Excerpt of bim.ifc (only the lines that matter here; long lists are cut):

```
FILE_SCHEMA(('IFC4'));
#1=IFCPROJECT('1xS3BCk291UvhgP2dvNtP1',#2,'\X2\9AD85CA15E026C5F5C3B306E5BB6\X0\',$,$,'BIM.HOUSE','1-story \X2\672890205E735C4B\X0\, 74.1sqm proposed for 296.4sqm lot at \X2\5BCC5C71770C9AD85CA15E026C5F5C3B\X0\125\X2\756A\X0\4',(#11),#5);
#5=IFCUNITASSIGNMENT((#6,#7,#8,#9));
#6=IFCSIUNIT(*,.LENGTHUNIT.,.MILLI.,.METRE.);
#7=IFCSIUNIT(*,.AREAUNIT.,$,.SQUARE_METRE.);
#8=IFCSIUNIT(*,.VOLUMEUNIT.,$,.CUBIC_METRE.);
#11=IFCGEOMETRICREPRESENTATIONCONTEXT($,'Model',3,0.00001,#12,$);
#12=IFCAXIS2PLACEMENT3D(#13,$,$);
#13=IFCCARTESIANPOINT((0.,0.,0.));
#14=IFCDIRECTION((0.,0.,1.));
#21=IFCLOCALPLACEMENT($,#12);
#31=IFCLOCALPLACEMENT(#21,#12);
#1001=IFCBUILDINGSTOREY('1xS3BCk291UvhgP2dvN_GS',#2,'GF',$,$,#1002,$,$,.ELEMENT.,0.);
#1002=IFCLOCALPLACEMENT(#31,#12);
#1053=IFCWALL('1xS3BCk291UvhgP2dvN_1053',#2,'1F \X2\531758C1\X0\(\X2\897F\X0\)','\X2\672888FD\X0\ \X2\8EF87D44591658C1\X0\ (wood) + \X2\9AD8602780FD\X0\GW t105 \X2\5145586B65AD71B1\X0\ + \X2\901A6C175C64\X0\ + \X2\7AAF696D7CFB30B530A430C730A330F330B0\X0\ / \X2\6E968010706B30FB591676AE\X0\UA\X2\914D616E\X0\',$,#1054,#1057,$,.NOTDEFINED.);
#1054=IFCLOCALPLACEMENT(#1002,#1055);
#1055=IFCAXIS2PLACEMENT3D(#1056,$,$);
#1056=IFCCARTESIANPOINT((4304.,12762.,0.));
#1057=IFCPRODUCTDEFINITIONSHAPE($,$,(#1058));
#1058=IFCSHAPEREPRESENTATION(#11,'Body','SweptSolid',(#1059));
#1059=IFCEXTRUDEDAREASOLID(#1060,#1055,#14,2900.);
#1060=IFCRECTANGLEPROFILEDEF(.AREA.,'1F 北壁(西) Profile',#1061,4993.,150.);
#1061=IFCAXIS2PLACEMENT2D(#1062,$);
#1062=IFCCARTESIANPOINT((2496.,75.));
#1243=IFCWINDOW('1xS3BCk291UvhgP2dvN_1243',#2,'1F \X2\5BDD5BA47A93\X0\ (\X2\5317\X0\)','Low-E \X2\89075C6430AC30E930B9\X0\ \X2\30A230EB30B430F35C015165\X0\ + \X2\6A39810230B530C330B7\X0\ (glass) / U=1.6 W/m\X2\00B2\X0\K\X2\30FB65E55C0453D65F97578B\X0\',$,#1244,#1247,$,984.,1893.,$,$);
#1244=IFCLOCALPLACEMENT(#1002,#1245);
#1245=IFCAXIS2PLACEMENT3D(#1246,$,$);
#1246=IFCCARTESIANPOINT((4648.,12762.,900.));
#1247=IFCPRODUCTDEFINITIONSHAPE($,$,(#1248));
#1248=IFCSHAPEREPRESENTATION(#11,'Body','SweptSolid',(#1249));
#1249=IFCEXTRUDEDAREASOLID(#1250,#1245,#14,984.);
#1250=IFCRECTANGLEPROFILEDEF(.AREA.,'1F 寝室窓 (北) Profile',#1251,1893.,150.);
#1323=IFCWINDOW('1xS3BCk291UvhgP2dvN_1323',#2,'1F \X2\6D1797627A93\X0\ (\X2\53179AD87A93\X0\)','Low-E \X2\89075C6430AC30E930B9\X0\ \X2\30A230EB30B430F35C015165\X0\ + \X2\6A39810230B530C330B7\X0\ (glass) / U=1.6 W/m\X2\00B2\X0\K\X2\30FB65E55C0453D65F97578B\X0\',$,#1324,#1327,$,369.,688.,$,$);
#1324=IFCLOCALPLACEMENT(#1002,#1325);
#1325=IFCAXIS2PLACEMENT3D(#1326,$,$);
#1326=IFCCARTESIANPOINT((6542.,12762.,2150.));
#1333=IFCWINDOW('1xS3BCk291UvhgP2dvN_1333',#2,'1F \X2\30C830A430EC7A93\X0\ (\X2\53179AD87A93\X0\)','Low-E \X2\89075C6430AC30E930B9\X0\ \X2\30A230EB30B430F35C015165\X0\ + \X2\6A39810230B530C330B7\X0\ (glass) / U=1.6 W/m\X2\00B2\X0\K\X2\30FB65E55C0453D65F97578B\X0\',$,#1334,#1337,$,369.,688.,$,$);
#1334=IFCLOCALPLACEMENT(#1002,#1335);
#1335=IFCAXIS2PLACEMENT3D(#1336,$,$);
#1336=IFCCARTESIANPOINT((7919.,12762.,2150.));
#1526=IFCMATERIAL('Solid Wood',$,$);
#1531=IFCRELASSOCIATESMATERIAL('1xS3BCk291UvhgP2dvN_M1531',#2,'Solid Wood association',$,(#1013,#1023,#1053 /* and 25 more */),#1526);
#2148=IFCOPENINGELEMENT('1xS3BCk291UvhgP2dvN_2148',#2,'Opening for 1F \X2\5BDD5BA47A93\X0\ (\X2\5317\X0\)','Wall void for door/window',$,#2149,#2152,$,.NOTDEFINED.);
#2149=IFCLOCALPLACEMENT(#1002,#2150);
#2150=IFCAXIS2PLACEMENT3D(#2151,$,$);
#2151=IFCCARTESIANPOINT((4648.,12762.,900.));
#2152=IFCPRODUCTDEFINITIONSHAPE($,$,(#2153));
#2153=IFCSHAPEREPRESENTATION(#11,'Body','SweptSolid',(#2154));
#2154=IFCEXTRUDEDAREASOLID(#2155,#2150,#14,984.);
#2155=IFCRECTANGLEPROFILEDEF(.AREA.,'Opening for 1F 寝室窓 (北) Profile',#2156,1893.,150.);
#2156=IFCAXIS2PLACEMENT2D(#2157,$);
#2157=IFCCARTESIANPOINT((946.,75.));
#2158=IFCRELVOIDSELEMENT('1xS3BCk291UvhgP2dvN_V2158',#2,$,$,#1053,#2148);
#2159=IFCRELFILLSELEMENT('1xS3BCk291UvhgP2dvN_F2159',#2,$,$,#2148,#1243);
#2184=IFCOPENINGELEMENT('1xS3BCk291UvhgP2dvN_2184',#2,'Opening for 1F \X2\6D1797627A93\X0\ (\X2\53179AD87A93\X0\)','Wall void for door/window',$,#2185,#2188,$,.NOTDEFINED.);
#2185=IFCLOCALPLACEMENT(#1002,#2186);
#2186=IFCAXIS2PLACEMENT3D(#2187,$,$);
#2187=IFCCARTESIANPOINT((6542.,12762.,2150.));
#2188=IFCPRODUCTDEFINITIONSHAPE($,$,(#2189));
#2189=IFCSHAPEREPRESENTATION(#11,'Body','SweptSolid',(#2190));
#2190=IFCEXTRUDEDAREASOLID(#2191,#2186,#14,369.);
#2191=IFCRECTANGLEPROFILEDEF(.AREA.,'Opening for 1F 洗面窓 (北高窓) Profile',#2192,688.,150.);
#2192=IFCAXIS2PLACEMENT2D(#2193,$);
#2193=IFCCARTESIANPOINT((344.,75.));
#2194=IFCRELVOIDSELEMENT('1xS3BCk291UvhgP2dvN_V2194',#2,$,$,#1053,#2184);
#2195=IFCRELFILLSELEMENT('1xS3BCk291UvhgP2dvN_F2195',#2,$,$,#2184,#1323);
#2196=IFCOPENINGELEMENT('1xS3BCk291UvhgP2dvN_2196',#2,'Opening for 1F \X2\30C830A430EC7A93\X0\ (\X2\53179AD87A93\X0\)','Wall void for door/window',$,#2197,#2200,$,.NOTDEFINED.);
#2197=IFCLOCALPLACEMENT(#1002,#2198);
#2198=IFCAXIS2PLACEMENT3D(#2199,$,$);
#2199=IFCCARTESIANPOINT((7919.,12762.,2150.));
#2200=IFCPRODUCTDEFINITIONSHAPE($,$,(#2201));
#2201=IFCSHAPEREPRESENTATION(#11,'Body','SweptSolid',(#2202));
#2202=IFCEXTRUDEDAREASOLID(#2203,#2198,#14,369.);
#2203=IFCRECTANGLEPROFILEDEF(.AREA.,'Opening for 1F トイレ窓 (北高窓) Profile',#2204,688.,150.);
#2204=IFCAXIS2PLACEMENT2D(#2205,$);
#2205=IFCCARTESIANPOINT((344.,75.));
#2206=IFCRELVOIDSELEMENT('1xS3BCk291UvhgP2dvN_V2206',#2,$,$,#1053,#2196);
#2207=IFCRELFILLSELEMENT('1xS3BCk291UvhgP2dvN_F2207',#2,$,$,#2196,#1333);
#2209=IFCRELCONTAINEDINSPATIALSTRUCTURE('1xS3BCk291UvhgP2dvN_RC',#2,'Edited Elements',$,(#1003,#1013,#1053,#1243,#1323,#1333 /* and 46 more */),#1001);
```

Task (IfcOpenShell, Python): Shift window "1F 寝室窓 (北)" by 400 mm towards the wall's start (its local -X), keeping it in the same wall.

```python
import ifcopenshell
import ifcopenshell.api.geometry
import ifcopenshell.util.placement
import ifcopenshell.util.unit

model = ifcopenshell.open("bim.ifc")
unit_scale = ifcopenshell.util.unit.calculate_unit_scale(model)

window = model.by_guid("1xS3BCk291UvhgP2dvN_1243")
opening = window.FillsVoids[0].RelatingOpeningElement
wall = opening.VoidsElements[0].RelatingBuildingElement

wall_matrix = ifcopenshell.util.placement.get_local_placement(wall.ObjectPlacement)
shift = wall_matrix[:3, 0] * -0.4 / unit_scale
before = ifcopenshell.util.placement.get_local_placement(window.ObjectPlacement)[:3, 3].copy()

# The window is not placed relative to its opening, so move both.
for product in (opening, window):
    matrix = ifcopenshell.util.placement.get_local_placement(product.ObjectPlacement)
    matrix[:3, 3] += shift
    ifcopenshell.api.geometry.edit_object_placement(model, product=product, matrix=matrix, is_si=False)

after = ifcopenshell.util.placement.get_local_placement(window.ObjectPlacement)[:3, 3]
print("window moved by", (after - before).round(3) + 0.0)

model.write("bim_updated.ifc")
```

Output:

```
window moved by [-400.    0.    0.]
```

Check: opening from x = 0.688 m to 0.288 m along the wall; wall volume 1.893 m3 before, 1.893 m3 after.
